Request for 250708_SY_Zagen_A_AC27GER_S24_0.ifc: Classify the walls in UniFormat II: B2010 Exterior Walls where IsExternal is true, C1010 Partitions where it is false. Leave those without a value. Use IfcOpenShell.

First a look at what the model holds.

```python
import ifcopenshell
import ifcopenshell.util.element

model = ifcopenshell.open("250708_SY_Zagen_A_AC27GER_S24_0.ifc")
print(model.schema)
print("classifications:", [c.Name for c in model.by_type("IfcClassification")])
values = [ifcopenshell.util.element.get_pset(e, "Pset_WallCommon", "IsExternal") for e in model.by_type("IfcWall")]
for value in (True, False, None):
    print("IsExternal", value, values.count(value))
```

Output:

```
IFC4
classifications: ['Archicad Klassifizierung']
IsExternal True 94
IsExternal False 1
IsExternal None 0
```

```python
import ifcopenshell
import ifcopenshell.api.classification
import ifcopenshell.util.element

model = ifcopenshell.open("250708_SY_Zagen_A_AC27GER_S24_0.ifc")

system = ifcopenshell.api.classification.add_classification(model, classification="UniFormat II")

walls = model.by_type("IfcWall")
external = {e: ifcopenshell.util.element.get_pset(e, "Pset_WallCommon", "IsExternal") for e in walls}
for flag, code, name in ((True, "B2010", "Exterior Walls"), (False, "C1010", "Partitions")):
    products = [e for e in walls if external[e] is flag]
    ifcopenshell.api.classification.add_reference(
        model, products=products, classification=system, identification=code, name=name
    )
    print(code, len(products))

model.write("250708_SY_Zagen_A_AC27GER_S24_0_v2.ifc")
```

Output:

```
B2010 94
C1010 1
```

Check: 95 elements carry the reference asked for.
